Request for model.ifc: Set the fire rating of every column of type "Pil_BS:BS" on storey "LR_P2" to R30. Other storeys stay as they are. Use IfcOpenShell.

First a look at what the model holds.

```python
import ifcopenshell
import ifcopenshell.util.element

model = ifcopenshell.open("model.ifc")
print(model.schema)
storey = next(s for s in model.by_type("IfcBuildingStorey") if s.Name == "LR_P2")
columns = [e for e in ifcopenshell.util.element.get_decomposition(storey) if e.is_a("IfcColumn")]
seen = {}
for e in columns:
    element_type = ifcopenshell.util.element.get_type(e)
    key = (element_type.Name if element_type != e and element_type else None, ifcopenshell.util.element.get_pset(e, "Pset_ColumnCommon", "FireRating"))
    seen[key] = seen.get(key, 0) + 1
for (name, value), count in sorted(seen.items(), key=str):
    print(count, "x", name, "|", value)
```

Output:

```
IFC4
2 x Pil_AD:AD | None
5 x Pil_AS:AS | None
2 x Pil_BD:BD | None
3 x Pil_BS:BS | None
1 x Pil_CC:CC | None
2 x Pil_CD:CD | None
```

```python
import ifcopenshell
import ifcopenshell.api.pset
import ifcopenshell.util.element

model = ifcopenshell.open("model.ifc")

storey = next(s for s in model.by_type("IfcBuildingStorey") if s.Name == "LR_P2")
columns = [e for e in ifcopenshell.util.element.get_decomposition(storey) if e.is_a("IfcColumn")]

count = 0
for e in columns:
    element_type = ifcopenshell.util.element.get_type(e)
    if element_type in (None, e) or element_type.Name != "Pil_BS:BS":
        continue
    # add_pset returns the element's existing set when there is one.
    pset = ifcopenshell.api.pset.add_pset(model, product=e, name="Pset_ColumnCommon")
    ifcopenshell.api.pset.edit_pset(model, pset=pset, properties={"FireRating": "R30"})
    count += 1

print(count, "columns updated")

model.write("model_edited.ifc")
```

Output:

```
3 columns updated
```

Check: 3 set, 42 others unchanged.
